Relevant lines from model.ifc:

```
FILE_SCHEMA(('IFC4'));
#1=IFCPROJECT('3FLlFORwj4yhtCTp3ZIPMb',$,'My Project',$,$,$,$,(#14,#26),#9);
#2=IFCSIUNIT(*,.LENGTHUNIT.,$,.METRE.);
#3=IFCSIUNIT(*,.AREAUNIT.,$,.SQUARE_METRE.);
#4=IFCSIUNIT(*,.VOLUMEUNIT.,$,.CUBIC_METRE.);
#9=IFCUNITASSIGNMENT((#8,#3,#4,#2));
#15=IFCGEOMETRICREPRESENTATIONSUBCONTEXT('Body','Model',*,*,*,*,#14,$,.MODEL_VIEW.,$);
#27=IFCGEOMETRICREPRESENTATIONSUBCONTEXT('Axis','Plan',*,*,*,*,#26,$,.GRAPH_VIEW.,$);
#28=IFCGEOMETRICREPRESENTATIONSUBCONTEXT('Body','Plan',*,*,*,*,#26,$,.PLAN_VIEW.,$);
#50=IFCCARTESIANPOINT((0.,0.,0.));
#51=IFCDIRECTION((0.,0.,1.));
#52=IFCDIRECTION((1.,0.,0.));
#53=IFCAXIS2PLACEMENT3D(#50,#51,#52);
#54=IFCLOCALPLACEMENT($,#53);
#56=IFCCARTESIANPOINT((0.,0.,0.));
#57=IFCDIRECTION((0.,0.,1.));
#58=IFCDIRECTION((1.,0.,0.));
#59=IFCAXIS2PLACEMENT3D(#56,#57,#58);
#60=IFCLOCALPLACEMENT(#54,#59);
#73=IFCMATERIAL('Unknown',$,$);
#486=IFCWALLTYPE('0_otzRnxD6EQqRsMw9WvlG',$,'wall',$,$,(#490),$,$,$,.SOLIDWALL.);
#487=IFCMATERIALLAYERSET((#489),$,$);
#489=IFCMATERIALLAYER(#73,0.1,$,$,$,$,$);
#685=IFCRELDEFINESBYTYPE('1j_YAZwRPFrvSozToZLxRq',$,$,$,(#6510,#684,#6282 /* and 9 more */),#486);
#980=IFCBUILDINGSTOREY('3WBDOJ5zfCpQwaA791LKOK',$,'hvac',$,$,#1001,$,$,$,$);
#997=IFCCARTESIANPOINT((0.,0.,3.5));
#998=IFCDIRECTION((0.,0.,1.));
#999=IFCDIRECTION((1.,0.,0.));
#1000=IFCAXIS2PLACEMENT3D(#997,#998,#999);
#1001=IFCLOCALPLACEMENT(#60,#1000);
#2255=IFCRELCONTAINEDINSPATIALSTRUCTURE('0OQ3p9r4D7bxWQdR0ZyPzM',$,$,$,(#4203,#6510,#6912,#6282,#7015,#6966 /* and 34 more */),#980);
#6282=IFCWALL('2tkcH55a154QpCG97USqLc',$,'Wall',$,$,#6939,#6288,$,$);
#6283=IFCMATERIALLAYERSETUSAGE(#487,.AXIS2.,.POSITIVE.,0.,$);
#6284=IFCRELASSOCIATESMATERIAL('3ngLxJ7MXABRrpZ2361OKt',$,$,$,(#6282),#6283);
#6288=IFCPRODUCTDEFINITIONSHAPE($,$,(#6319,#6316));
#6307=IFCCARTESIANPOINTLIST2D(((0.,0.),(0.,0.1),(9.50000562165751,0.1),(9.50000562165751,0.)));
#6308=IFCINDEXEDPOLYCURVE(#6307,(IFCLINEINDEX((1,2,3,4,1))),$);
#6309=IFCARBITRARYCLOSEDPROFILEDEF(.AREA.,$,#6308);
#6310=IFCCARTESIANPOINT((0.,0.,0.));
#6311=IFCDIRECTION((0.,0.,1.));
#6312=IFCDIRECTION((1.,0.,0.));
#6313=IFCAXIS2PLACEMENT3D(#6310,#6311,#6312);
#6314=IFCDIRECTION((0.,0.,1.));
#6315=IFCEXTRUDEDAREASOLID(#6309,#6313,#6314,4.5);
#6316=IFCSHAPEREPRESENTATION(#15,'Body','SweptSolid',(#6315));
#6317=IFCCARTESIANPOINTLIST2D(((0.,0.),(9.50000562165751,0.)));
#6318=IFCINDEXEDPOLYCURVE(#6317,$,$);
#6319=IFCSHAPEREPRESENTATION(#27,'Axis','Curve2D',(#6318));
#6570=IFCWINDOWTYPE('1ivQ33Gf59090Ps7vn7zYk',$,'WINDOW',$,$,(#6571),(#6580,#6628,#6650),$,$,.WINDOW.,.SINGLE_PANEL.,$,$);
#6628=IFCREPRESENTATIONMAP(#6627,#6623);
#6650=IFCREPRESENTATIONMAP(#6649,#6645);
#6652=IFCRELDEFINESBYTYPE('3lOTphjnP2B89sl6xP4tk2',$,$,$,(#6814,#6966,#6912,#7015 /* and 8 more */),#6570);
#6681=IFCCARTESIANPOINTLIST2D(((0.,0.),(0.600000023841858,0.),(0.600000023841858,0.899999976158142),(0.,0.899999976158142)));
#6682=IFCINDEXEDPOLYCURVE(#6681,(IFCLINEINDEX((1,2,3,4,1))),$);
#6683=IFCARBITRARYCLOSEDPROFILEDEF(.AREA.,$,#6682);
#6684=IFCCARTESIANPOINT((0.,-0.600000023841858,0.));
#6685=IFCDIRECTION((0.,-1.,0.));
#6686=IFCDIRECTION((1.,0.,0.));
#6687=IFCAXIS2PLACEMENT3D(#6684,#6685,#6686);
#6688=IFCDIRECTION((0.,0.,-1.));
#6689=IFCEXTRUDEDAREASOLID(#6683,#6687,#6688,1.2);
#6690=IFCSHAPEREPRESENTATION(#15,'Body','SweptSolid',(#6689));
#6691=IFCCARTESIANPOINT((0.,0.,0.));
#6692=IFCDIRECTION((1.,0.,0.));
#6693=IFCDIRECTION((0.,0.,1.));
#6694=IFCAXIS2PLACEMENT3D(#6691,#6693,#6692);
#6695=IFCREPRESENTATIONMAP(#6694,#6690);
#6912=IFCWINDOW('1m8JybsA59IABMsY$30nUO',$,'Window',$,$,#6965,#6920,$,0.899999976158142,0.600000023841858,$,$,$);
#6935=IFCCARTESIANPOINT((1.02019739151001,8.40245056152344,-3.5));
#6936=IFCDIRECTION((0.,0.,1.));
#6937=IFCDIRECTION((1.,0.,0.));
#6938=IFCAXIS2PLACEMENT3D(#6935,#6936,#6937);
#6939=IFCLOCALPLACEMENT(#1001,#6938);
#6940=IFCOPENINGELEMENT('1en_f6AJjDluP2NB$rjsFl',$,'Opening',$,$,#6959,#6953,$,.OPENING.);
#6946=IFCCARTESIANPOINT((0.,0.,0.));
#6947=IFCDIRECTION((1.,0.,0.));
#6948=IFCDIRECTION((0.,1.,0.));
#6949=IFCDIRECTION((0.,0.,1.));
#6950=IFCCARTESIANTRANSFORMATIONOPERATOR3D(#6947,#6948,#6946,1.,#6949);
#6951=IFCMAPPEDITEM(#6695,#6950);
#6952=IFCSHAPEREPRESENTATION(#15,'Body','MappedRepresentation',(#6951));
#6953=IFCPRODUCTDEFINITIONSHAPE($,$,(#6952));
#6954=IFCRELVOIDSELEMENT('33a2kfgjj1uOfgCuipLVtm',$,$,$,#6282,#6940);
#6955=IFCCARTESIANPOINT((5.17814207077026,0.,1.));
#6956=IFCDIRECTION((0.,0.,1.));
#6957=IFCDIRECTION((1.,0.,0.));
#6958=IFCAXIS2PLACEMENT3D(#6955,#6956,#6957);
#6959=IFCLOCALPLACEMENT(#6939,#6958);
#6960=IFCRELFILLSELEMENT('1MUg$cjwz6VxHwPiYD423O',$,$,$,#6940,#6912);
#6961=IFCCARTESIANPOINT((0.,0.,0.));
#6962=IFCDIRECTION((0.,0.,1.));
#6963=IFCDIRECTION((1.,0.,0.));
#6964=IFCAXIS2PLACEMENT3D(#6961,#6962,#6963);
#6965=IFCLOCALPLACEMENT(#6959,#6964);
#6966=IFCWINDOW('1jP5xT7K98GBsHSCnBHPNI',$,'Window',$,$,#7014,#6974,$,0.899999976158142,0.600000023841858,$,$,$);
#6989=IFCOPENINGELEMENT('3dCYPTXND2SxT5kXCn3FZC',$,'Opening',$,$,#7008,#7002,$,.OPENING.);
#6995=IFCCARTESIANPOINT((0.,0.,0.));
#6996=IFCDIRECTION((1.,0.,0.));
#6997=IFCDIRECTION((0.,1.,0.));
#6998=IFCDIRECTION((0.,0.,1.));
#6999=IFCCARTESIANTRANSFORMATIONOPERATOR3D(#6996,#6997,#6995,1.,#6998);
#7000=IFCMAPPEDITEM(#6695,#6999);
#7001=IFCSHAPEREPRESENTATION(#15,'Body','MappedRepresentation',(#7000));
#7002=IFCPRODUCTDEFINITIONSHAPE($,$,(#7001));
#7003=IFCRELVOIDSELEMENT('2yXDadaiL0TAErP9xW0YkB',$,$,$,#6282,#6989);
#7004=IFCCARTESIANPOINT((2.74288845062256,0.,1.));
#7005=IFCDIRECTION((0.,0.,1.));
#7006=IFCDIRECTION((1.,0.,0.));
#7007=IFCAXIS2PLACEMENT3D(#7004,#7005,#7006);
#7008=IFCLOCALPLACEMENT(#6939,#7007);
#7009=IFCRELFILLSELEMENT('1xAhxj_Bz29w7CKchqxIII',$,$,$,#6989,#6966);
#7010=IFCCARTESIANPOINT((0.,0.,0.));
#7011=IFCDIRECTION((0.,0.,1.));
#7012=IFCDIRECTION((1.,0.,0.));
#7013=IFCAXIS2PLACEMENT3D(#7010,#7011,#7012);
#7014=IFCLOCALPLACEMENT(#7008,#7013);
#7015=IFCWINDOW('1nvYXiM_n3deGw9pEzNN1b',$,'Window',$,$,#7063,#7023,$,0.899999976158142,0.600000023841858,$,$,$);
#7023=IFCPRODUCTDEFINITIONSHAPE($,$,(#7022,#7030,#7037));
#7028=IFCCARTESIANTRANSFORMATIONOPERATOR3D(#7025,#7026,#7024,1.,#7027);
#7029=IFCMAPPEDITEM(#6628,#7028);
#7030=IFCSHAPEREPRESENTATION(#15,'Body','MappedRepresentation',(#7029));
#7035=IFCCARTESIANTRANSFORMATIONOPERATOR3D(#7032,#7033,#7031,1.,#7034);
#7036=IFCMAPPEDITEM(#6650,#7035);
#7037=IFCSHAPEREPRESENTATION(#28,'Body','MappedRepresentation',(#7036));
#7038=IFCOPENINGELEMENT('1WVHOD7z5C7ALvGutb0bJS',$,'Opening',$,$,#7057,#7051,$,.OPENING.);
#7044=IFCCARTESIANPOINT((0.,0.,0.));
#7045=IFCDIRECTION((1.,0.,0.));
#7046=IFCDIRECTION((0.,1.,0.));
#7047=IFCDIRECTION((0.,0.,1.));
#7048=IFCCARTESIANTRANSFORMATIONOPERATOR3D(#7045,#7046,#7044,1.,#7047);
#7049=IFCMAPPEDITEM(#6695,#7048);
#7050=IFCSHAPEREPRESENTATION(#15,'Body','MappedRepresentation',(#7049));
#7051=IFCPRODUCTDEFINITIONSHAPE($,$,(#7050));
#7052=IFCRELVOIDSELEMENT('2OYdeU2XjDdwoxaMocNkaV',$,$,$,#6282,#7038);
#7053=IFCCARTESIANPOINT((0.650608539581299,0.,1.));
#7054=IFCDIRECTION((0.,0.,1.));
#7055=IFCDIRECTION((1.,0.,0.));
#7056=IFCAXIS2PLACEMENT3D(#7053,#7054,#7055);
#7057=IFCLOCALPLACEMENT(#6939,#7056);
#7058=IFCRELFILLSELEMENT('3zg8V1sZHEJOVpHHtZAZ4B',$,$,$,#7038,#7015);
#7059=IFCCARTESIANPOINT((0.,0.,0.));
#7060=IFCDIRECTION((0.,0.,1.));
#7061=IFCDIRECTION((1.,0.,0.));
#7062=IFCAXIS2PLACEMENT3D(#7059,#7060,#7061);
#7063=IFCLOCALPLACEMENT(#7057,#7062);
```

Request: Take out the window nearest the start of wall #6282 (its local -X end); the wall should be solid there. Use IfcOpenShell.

```python
import ifcopenshell
import ifcopenshell.api.feature
import ifcopenshell.api.root
import ifcopenshell.geom
import ifcopenshell.util.shape

model = ifcopenshell.open("model.ifc")
settings = ifcopenshell.geom.settings()


def volume(element):
    """Net volume in cubic metres, openings subtracted."""
    shape = ifcopenshell.geom.create_shape(settings, element)
    return ifcopenshell.util.shape.get_volume(shape.geometry)


window = model.by_guid("1nvYXiM_n3deGw9pEzNN1b")
opening = window.FillsVoids[0].RelatingOpeningElement
wall = opening.VoidsElements[0].RelatingBuildingElement
before = volume(wall)

ifcopenshell.api.root.remove_product(model, product=window)
ifcopenshell.api.feature.remove_feature(model, feature=opening)

after = volume(wall)

print(f"wall volume {before:.3f} -> {after:.3f} m3")

model.write("model_rev.ifc")
```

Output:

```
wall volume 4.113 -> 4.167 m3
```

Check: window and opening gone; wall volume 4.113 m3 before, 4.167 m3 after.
